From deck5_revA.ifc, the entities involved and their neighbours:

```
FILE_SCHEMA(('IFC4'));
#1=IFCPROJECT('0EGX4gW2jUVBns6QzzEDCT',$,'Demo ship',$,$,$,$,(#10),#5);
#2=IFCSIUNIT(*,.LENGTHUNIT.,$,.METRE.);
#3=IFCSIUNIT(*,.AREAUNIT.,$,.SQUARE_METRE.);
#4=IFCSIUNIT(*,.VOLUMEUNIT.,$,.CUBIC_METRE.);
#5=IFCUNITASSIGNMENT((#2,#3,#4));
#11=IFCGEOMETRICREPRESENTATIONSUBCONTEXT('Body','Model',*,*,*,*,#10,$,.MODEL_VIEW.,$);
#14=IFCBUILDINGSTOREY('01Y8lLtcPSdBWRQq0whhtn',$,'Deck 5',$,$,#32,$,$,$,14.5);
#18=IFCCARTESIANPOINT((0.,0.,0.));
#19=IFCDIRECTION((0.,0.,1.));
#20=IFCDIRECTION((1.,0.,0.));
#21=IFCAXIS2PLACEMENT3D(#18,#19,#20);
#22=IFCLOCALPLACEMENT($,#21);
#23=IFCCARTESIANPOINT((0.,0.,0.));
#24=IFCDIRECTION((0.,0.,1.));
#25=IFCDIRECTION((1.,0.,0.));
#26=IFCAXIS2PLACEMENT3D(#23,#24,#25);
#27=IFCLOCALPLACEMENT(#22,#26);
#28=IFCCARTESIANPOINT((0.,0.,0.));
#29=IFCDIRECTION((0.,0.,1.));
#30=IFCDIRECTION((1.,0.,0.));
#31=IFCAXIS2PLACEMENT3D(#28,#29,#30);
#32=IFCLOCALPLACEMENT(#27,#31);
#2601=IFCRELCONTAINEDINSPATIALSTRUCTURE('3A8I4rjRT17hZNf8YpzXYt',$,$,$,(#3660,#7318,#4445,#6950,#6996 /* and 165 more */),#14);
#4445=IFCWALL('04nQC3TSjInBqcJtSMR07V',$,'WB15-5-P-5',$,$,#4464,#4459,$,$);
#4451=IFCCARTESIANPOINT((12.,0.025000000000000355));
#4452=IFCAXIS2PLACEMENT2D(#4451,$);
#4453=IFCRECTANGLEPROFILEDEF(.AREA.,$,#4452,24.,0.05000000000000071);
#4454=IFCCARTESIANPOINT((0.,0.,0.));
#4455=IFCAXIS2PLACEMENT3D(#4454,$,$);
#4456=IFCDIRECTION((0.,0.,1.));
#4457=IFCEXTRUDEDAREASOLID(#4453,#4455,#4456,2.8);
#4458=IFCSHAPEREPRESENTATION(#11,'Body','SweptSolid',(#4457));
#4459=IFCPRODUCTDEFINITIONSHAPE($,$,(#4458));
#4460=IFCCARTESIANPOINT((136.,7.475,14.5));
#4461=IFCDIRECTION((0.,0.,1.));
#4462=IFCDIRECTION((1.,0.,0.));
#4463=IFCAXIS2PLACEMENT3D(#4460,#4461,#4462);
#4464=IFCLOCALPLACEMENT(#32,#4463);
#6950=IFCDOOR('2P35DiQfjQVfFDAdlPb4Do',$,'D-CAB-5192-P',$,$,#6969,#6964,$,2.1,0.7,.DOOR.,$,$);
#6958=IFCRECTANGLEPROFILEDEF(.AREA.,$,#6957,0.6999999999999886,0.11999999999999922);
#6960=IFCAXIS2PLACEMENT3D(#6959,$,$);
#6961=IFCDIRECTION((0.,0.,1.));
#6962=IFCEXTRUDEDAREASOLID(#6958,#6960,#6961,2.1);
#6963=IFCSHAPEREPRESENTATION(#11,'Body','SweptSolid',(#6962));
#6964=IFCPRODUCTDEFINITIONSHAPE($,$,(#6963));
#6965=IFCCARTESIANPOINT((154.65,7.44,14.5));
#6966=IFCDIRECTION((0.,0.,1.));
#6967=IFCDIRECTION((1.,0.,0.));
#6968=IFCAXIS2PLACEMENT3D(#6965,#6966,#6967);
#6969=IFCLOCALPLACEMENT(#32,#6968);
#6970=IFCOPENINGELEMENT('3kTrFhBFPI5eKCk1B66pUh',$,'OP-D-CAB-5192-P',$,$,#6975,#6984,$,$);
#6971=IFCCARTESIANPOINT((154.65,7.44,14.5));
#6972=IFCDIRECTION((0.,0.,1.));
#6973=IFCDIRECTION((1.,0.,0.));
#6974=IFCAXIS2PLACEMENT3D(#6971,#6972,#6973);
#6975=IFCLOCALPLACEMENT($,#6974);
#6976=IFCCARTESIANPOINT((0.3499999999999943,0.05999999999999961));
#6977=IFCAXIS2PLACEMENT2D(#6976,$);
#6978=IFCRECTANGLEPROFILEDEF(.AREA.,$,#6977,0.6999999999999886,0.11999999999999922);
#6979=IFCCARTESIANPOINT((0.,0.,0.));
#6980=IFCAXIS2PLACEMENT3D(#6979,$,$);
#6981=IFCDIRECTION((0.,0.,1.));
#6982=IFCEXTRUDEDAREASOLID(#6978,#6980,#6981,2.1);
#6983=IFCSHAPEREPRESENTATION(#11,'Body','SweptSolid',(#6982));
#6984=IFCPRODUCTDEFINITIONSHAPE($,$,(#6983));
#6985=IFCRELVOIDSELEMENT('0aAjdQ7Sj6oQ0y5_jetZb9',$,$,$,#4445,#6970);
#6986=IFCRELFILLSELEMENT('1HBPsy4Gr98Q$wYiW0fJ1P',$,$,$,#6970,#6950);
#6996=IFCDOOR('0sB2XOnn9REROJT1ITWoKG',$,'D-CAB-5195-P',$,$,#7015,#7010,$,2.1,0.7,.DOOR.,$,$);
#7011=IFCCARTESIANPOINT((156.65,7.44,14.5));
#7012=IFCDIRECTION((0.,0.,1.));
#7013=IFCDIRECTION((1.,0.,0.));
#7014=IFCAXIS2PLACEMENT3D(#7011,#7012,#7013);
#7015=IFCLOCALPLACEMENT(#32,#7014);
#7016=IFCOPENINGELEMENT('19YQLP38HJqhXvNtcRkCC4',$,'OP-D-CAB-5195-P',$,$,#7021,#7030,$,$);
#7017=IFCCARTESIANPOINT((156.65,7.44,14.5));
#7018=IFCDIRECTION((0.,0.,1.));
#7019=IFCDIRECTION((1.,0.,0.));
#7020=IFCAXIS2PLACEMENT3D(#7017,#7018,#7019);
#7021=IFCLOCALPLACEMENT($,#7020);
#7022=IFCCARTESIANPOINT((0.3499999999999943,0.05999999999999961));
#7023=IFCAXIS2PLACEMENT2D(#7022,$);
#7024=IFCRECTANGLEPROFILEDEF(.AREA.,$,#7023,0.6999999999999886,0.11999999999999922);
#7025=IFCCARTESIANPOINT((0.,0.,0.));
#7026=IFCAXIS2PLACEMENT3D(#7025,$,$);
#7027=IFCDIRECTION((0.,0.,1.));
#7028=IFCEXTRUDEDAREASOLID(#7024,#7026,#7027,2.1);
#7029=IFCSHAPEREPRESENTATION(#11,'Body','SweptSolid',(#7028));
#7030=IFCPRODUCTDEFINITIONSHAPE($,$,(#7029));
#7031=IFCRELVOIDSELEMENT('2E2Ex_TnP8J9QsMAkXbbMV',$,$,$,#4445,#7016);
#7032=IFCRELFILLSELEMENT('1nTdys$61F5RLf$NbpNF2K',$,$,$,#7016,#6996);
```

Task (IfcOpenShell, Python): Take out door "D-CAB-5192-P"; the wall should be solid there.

```python
import ifcopenshell
import ifcopenshell.api.feature
import ifcopenshell.api.root
import ifcopenshell.geom
import ifcopenshell.util.shape

model = ifcopenshell.open("deck5_revA.ifc")
settings = ifcopenshell.geom.settings()


def volume(element):
    """Net volume in cubic metres, openings subtracted."""
    shape = ifcopenshell.geom.create_shape(settings, element)
    return ifcopenshell.util.shape.get_volume(shape.geometry)


door = model.by_guid("2P35DiQfjQVfFDAdlPb4Do")
opening = door.FillsVoids[0].RelatingOpeningElement
wall = opening.VoidsElements[0].RelatingBuildingElement
before = volume(wall)

ifcopenshell.api.root.remove_product(model, product=door)
ifcopenshell.api.feature.remove_feature(model, feature=opening)

after = volume(wall)

print(f"wall volume {before:.3f} -> {after:.3f} m3")

model.write("deck5_revA_edited.ifc")
```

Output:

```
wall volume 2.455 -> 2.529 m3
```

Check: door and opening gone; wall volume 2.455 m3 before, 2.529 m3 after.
